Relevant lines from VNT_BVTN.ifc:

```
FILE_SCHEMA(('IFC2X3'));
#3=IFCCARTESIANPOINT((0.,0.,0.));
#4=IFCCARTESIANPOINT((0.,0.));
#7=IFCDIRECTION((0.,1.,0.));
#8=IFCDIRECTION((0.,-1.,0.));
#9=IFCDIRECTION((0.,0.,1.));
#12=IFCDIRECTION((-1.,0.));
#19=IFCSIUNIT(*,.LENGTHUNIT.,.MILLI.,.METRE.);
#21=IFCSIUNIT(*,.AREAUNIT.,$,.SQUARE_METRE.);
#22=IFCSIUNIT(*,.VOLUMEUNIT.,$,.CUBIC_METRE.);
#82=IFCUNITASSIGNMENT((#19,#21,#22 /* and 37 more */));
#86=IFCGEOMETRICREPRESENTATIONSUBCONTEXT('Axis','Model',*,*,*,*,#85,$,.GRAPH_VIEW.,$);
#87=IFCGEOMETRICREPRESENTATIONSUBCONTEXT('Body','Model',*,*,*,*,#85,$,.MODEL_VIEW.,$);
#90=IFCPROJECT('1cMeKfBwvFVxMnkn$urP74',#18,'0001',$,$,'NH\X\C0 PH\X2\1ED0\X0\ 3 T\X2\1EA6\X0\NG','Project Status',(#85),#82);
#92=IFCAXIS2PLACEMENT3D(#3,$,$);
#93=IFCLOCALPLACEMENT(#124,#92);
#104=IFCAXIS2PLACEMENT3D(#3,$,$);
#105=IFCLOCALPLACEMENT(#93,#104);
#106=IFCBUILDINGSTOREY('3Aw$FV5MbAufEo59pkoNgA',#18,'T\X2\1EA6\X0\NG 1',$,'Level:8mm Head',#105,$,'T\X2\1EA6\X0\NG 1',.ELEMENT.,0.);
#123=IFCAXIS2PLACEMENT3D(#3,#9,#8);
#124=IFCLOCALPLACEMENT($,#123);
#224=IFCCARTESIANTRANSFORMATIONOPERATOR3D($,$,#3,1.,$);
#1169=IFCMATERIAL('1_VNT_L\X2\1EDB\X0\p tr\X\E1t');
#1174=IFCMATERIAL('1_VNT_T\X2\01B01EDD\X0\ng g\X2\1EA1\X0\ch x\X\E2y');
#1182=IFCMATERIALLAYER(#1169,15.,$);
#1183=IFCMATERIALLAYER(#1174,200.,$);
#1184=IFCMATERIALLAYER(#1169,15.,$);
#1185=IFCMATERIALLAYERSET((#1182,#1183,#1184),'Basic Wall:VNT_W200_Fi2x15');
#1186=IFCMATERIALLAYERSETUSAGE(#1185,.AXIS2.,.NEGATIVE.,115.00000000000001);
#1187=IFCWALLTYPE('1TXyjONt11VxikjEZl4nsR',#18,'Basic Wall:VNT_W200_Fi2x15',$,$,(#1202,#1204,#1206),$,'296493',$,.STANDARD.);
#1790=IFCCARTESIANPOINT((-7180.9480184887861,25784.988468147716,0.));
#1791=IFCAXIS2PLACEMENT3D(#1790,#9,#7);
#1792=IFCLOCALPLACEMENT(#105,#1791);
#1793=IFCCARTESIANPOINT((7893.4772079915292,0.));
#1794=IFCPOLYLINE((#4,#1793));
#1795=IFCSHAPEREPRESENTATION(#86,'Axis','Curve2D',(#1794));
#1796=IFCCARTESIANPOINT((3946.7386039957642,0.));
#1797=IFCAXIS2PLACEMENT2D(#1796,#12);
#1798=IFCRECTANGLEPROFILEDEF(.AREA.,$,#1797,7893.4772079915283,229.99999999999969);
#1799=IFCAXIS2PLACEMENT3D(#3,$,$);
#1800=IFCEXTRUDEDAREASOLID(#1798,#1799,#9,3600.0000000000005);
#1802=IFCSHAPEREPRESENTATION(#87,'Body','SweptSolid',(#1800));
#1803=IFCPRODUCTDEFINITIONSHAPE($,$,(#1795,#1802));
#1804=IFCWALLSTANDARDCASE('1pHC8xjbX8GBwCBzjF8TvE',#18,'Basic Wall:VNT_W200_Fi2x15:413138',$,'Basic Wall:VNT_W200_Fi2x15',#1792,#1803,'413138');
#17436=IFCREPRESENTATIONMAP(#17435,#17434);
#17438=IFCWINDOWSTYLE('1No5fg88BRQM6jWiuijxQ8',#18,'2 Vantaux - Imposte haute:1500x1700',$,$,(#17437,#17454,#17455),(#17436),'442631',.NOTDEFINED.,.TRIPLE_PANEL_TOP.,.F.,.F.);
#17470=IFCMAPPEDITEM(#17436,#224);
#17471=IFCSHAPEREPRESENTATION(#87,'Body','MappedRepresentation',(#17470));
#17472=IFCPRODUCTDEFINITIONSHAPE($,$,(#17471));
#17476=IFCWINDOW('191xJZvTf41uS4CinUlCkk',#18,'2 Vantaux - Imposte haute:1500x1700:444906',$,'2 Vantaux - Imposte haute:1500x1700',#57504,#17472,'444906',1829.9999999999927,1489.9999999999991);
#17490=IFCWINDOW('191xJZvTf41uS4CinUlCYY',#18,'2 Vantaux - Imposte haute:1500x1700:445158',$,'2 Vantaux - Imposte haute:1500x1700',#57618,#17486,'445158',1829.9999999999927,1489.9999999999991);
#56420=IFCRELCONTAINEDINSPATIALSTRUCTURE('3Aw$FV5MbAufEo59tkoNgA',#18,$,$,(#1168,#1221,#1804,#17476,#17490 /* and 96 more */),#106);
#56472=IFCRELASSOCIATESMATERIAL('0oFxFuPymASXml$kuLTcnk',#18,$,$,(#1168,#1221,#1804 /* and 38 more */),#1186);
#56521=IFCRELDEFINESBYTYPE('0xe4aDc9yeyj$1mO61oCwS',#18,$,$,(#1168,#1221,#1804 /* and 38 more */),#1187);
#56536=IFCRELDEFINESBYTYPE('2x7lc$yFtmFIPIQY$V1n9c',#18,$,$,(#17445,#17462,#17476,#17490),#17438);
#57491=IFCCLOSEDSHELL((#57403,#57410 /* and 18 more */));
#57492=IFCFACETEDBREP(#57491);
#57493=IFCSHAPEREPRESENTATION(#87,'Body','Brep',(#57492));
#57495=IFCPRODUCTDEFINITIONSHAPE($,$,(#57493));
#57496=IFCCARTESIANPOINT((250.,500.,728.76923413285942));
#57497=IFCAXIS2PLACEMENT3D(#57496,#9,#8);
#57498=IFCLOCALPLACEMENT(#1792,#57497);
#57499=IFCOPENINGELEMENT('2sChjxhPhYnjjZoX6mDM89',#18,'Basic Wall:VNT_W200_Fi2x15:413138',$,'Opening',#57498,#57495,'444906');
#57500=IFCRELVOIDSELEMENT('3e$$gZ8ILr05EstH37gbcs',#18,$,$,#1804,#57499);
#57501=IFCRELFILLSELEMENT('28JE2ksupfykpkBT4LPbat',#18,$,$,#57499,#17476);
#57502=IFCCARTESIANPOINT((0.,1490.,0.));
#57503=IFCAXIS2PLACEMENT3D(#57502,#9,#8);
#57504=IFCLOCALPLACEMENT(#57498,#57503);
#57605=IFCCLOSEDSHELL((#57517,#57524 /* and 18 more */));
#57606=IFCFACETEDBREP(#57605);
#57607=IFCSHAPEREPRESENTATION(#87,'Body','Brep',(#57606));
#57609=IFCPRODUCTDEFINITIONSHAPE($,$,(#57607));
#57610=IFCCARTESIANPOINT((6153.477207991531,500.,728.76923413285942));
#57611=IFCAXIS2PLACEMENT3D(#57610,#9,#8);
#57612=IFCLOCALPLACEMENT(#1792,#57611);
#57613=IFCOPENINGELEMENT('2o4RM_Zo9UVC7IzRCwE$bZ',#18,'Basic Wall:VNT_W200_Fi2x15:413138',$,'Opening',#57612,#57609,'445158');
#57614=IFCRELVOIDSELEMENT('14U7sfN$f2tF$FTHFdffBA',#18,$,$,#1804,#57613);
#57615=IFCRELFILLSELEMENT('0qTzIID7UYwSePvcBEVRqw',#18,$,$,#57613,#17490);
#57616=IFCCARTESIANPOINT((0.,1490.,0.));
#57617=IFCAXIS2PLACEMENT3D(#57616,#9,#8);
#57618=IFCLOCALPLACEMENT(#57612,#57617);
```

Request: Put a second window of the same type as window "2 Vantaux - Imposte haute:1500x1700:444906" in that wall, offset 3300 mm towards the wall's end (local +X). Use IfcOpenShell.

```python
import ifcopenshell
import ifcopenshell.api.feature
import ifcopenshell.api.geometry
import ifcopenshell.api.root
import ifcopenshell.geom
import ifcopenshell.util.element
import ifcopenshell.util.placement
import ifcopenshell.util.shape

model = ifcopenshell.open("VNT_BVTN.ifc")
settings = ifcopenshell.geom.settings()


def volume(element):
    """Net volume in cubic metres, openings subtracted."""
    shape = ifcopenshell.geom.create_shape(settings, element)
    return ifcopenshell.util.shape.get_volume(shape.geometry)


def reuse_history(source, copy):
    """copy_class also copies each property set's owner history, people and application; keep the originals."""
    for rel in copy.IsDefinedBy:
        if rel.is_a("IfcRelDefinesByProperties") and (history := rel.RelatingPropertyDefinition.OwnerHistory):
            rel.RelatingPropertyDefinition.OwnerHistory = source.OwnerHistory
            ifcopenshell.util.element.remove_deep2(model, history)


window = model.by_guid("191xJZvTf41uS4CinUlCkk")
opening = window.FillsVoids[0].RelatingOpeningElement
wall = opening.VoidsElements[0].RelatingBuildingElement
before = volume(wall)
shift = ifcopenshell.util.placement.get_local_placement(wall.ObjectPlacement)[:3, 0] * 3300.0

# copy_class copies the void relationship, type, container and properties, but no geometry.
new_opening = ifcopenshell.api.root.copy_class(model, product=opening)
new_opening.Representation = ifcopenshell.util.element.copy_deep(
    model, opening.Representation, exclude=["IfcGeometricRepresentationContext", "IfcRepresentationMap"]
)
new_opening.Name = "Basic Wall:VNT_W200_Fi2x15"
new_opening.Tag = None
new_window = ifcopenshell.api.root.copy_class(model, product=window)
new_window.Representation = ifcopenshell.util.element.copy_deep(
    model, window.Representation, exclude=["IfcGeometricRepresentationContext", "IfcRepresentationMap"]
)
new_window.Name = "2 Vantaux - Imposte haute:1500x1700"
new_window.Tag = None
reuse_history(window, new_window)
fills = ifcopenshell.api.feature.add_filling(model, opening=new_opening, element=new_window)
fills.OwnerHistory = new_window.OwnerHistory  # required in IFC2X3

for old, new in ((opening, new_opening), (window, new_window)):
    matrix = ifcopenshell.util.placement.get_local_placement(old.ObjectPlacement)
    matrix[:3, 3] += shift
    ifcopenshell.api.geometry.edit_object_placement(model, product=new, matrix=matrix, is_si=False)

after = volume(wall)

print(f"wall volume {before:.3f} -> {after:.3f} m3")

model.write("VNT_BVTN_rev.ifc")
```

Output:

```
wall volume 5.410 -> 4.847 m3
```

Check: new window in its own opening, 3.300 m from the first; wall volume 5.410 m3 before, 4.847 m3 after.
